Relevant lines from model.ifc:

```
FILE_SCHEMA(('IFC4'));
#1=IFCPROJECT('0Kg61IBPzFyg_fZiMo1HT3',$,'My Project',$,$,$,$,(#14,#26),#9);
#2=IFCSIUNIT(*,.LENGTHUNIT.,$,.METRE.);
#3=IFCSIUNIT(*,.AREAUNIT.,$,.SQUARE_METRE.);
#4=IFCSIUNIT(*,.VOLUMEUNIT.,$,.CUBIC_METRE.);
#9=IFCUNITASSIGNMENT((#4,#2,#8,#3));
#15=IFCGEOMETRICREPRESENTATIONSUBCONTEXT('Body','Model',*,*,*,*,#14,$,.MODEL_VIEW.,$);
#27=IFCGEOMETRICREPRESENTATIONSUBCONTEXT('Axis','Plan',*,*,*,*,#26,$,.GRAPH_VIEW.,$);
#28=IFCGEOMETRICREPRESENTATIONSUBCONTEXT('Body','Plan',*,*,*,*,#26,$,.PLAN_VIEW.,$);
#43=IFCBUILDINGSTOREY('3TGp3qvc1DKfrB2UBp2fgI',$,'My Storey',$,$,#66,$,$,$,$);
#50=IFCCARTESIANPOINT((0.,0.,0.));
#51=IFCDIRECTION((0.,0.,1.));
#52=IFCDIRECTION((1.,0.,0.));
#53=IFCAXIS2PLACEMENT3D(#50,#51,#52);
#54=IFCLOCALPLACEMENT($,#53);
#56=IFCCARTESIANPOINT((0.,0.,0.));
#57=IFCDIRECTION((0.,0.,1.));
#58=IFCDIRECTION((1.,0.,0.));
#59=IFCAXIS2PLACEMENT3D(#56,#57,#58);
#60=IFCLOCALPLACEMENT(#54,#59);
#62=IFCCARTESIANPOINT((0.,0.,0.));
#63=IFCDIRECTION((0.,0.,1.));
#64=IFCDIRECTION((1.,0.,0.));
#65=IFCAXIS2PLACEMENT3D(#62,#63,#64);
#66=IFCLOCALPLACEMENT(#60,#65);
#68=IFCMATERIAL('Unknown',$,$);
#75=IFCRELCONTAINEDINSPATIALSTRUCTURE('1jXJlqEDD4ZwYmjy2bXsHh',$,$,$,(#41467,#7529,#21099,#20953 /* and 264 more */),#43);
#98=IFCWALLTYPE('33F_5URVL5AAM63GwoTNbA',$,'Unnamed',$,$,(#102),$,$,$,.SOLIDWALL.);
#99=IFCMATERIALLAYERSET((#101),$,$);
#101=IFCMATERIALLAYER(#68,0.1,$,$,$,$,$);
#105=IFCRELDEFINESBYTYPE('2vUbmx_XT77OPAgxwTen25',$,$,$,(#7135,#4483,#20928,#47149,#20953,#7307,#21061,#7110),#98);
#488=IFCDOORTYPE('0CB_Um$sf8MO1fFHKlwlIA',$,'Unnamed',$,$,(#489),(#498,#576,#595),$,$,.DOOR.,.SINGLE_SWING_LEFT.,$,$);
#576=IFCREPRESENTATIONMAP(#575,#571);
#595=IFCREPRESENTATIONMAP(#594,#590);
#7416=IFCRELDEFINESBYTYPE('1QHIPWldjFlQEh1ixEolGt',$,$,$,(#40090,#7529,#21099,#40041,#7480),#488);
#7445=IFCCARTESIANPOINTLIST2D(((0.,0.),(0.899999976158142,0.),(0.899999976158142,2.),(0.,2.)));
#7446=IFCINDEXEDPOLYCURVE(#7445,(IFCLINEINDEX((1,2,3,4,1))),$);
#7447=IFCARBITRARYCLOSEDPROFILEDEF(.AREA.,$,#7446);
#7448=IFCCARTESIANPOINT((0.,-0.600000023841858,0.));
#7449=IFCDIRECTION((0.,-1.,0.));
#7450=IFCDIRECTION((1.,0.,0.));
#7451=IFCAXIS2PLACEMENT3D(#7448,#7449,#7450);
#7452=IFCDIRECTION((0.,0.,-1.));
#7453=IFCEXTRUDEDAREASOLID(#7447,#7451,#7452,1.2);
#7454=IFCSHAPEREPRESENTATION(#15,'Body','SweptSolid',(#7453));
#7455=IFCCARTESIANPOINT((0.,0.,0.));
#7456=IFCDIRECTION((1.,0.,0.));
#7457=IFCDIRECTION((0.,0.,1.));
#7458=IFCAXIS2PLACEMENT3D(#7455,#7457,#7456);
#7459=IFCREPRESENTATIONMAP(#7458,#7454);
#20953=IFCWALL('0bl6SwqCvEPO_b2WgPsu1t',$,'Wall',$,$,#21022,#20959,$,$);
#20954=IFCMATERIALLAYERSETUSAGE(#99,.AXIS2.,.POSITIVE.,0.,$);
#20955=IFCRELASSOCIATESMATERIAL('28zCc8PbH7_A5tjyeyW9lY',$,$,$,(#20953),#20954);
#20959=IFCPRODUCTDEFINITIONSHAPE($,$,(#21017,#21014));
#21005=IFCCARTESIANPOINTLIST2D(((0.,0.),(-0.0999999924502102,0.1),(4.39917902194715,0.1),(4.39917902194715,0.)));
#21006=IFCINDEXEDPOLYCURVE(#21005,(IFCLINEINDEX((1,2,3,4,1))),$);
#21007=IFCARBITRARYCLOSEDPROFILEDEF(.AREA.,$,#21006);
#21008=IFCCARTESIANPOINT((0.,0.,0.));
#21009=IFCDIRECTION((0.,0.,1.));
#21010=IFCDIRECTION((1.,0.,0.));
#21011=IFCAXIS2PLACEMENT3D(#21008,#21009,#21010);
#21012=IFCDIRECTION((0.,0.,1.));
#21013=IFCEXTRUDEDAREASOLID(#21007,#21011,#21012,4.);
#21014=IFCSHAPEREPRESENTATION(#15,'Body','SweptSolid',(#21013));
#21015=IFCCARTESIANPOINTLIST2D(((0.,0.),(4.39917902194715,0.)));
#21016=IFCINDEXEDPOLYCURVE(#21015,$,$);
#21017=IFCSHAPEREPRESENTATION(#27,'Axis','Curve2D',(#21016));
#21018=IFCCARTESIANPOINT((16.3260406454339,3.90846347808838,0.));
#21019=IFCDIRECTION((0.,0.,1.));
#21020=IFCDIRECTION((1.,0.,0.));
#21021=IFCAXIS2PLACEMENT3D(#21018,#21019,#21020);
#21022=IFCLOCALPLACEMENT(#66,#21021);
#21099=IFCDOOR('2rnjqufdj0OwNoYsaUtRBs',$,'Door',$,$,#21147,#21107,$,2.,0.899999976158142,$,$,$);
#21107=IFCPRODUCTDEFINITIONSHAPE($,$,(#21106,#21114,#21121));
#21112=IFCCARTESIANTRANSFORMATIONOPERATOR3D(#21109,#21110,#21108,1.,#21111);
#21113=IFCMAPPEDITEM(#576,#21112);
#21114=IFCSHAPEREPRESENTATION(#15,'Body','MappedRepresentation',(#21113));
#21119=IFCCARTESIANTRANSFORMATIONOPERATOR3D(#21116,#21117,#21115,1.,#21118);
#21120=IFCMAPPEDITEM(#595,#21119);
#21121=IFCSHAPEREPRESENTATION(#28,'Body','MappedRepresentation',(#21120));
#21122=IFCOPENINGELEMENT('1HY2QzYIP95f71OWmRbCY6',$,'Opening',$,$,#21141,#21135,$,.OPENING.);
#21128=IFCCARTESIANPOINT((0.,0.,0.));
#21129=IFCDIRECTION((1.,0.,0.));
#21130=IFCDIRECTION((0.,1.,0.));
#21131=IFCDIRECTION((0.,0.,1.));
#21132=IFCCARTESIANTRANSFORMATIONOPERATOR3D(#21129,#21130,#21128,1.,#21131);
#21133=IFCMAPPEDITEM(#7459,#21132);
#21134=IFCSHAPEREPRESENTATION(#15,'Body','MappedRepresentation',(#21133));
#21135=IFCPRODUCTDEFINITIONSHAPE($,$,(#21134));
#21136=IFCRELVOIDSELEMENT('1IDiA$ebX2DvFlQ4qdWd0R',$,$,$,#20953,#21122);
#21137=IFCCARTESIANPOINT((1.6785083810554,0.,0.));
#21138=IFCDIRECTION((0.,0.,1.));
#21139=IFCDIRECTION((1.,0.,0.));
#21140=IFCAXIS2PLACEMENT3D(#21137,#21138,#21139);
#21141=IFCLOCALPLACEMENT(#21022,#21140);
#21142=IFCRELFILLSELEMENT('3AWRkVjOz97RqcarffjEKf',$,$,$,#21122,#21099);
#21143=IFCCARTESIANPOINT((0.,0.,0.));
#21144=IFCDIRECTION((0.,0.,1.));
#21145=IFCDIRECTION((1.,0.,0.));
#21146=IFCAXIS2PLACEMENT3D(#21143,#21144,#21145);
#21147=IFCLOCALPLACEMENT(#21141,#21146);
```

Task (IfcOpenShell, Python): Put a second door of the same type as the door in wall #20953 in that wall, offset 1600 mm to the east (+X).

```python
import ifcopenshell
import ifcopenshell.api.feature
import ifcopenshell.api.geometry
import ifcopenshell.api.root
import ifcopenshell.geom
import ifcopenshell.util.element
import ifcopenshell.util.placement
import ifcopenshell.util.shape
import ifcopenshell.util.unit

model = ifcopenshell.open("model.ifc")
unit_scale = ifcopenshell.util.unit.calculate_unit_scale(model)
settings = ifcopenshell.geom.settings()


def volume(element):
    """Net volume in cubic metres, openings subtracted."""
    shape = ifcopenshell.geom.create_shape(settings, element)
    return ifcopenshell.util.shape.get_volume(shape.geometry)


door = model.by_id(21099)
opening = door.FillsVoids[0].RelatingOpeningElement
wall = opening.VoidsElements[0].RelatingBuildingElement
before = volume(wall)
shift = ifcopenshell.util.placement.get_local_placement(wall.ObjectPlacement)[:3, 0] * 1.6 / unit_scale

# copy_class copies the void relationship, type, container and properties, but no geometry.
new_opening = ifcopenshell.api.root.copy_class(model, product=opening)
new_opening.Representation = ifcopenshell.util.element.copy_deep(
    model, opening.Representation, exclude=["IfcGeometricRepresentationContext", "IfcRepresentationMap"]
)
new_door = ifcopenshell.api.root.copy_class(model, product=door)
new_door.Representation = ifcopenshell.util.element.copy_deep(
    model, door.Representation, exclude=["IfcGeometricRepresentationContext", "IfcRepresentationMap"]
)
ifcopenshell.api.feature.add_filling(model, opening=new_opening, element=new_door)

for old, new in ((opening, new_opening), (door, new_door)):
    matrix = ifcopenshell.util.placement.get_local_placement(old.ObjectPlacement)
    matrix[:3, 3] += shift
    ifcopenshell.api.geometry.edit_object_placement(model, product=new, matrix=matrix, is_si=False)

after = volume(wall)

print(f"wall volume {before:.3f} -> {after:.3f} m3")

model.write("model_edited.ifc")
```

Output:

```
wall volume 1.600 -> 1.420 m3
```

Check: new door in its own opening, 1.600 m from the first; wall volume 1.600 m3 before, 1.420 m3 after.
